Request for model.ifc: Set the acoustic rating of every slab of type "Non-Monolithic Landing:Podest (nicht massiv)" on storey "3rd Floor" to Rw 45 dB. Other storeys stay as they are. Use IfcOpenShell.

First a look at what the model holds.

```python
import ifcopenshell
import ifcopenshell.util.element

model = ifcopenshell.open("model.ifc")
print(model.schema)
storey = next(s for s in model.by_type("IfcBuildingStorey") if s.Name == "3rd Floor")
slabs = [e for e in ifcopenshell.util.element.get_decomposition(storey) if e.is_a("IfcSlab")]
seen = {}
for e in slabs:
    element_type = ifcopenshell.util.element.get_type(e)
    key = (element_type.Name if element_type != e and element_type else None, ifcopenshell.util.element.get_pset(e, "Pset_SlabCommon", "AcousticRating"))
    seen[key] = seen.get(key, 0) + 1
for (name, value), count in sorted(seen.items(), key=str):
    print(count, "x", name, "|", value)
```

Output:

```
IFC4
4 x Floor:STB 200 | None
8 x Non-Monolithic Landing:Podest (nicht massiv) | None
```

```python
import ifcopenshell
import ifcopenshell.api.pset
import ifcopenshell.util.element

model = ifcopenshell.open("model.ifc")

storey = next(s for s in model.by_type("IfcBuildingStorey") if s.Name == "3rd Floor")
slabs = [e for e in ifcopenshell.util.element.get_decomposition(storey) if e.is_a("IfcSlab")]

count = 0
for e in slabs:
    element_type = ifcopenshell.util.element.get_type(e)
    if element_type in (None, e) or element_type.Name != "Non-Monolithic Landing:Podest (nicht massiv)":
        continue
    # add_pset returns the element's existing set when there is one.
    pset = ifcopenshell.api.pset.add_pset(model, product=e, name="Pset_SlabCommon")
    ifcopenshell.api.pset.edit_pset(model, pset=pset, properties={"AcousticRating": "Rw 45 dB"})
    count += 1

print(count, "slabs updated")

model.write("model_rev.ifc")
```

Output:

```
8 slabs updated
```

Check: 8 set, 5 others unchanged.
